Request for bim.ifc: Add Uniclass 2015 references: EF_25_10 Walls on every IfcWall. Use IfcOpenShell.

First a look at what the model holds.

```python
import ifcopenshell

model = ifcopenshell.open("bim.ifc")
print(model.schema)
print("classifications:", [c.Name for c in model.by_type("IfcClassification")])
for ifc_class in ("IfcDoor", "IfcRoof", "IfcStair", "IfcWall", "IfcWindow"):
    print(ifc_class, len(model.by_type(ifc_class)))
```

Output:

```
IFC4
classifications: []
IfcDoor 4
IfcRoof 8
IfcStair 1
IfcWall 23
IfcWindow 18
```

```python
import ifcopenshell
import ifcopenshell.api.classification

model = ifcopenshell.open("bim.ifc")

system = ifcopenshell.api.classification.add_classification(model, classification="Uniclass 2015")

codes = {
    "IfcWall": ("EF_25_10", "Walls"),
}
for ifc_class, (code, name) in codes.items():
    products = model.by_type(ifc_class)
    ifcopenshell.api.classification.add_reference(
        model, products=products, classification=system, identification=code, name=name
    )
    print(code, len(products))

model.write("bim-out.ifc")
```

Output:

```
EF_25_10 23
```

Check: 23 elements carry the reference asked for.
